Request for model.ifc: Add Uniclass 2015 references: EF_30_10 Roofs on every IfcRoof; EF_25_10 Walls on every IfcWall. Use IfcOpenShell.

First a look at what the model holds.

```python
import ifcopenshell

model = ifcopenshell.open("model.ifc")
print(model.schema)
print("classifications:", [c.Name for c in model.by_type("IfcClassification")])
for ifc_class in ("IfcDoor", "IfcRoof", "IfcStair", "IfcWall", "IfcWindow"):
    print(ifc_class, len(model.by_type(ifc_class)))
```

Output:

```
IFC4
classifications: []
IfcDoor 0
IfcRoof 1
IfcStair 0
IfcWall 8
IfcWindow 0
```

```python
import ifcopenshell
import ifcopenshell.api.classification

model = ifcopenshell.open("model.ifc")

system = ifcopenshell.api.classification.add_classification(model, classification="Uniclass 2015")

codes = {
    "IfcRoof": ("EF_30_10", "Roofs"),
    "IfcWall": ("EF_25_10", "Walls"),
}
for ifc_class, (code, name) in codes.items():
    products = model.by_type(ifc_class)
    ifcopenshell.api.classification.add_reference(
        model, products=products, classification=system, identification=code, name=name
    )
    print(code, len(products))

model.write("model-out.ifc")
```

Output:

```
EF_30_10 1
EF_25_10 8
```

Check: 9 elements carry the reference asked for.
